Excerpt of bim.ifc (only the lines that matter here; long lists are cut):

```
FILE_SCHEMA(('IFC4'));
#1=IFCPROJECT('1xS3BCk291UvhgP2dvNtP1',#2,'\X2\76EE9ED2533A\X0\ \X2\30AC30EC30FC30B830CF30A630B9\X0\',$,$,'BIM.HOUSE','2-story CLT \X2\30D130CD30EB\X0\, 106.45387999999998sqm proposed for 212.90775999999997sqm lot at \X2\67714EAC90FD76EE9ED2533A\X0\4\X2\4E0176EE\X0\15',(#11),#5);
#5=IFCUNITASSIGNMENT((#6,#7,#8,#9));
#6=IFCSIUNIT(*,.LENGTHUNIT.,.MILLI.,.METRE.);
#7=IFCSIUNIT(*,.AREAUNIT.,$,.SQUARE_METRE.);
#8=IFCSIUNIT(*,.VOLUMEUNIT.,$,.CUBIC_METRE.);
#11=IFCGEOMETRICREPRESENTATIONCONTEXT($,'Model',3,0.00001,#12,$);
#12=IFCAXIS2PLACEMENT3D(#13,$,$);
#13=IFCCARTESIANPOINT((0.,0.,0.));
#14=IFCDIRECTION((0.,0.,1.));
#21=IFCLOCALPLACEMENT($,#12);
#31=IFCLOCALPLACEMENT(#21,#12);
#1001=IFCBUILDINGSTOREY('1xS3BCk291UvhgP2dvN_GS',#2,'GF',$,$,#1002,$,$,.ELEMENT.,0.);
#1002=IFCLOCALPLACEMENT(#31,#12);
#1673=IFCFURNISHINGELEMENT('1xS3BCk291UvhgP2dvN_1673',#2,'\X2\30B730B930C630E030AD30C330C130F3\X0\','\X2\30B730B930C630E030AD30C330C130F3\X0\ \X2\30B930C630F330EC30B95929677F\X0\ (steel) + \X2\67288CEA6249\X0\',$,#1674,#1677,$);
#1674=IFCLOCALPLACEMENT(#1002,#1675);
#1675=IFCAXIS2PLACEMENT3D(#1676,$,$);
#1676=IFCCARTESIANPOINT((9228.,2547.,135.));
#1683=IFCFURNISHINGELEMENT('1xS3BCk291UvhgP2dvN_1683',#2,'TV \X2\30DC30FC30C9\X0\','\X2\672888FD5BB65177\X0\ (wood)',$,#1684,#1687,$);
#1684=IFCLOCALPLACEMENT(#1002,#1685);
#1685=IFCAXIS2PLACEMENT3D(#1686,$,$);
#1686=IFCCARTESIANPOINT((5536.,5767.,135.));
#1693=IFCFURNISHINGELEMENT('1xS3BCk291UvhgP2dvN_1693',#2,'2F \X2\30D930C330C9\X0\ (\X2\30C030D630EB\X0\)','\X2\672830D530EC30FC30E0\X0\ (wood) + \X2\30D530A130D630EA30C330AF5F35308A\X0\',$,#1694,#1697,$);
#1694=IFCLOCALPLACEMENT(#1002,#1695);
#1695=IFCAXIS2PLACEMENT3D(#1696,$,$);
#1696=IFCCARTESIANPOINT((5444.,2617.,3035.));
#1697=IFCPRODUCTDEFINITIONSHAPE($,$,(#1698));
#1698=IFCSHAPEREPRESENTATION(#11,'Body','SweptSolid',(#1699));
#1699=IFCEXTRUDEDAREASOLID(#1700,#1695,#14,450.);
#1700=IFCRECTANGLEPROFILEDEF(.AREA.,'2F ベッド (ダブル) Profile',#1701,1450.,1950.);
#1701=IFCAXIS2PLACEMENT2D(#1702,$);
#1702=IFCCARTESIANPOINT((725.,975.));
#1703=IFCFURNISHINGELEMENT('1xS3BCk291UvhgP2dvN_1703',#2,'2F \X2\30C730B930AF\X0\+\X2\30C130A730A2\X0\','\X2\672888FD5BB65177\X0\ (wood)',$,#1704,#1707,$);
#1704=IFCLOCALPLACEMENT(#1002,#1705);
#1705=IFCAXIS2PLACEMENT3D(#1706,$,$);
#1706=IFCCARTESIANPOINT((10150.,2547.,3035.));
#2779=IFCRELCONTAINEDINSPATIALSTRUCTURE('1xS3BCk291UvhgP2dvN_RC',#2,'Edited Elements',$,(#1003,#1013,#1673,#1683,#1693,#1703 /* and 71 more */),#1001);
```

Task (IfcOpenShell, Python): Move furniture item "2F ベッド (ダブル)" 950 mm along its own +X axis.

```python
import ifcopenshell
import ifcopenshell.api.geometry
import ifcopenshell.util.placement

model = ifcopenshell.open("bim.ifc")

item = model.by_guid("1xS3BCk291UvhgP2dvN_1693")
matrix = ifcopenshell.util.placement.get_local_placement(item.ObjectPlacement)
matrix[:3, 3] += matrix[:3, 0] * 950.0
ifcopenshell.api.geometry.edit_object_placement(model, product=item, matrix=matrix, is_si=False)

print(ifcopenshell.util.placement.get_local_placement(item.ObjectPlacement).round(3) + 0.0)

model.write("bim_updated.ifc")
```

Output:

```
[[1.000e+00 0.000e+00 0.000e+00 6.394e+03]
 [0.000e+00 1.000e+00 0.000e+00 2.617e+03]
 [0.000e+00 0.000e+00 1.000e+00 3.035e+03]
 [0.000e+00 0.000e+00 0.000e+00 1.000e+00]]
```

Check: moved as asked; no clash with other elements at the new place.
